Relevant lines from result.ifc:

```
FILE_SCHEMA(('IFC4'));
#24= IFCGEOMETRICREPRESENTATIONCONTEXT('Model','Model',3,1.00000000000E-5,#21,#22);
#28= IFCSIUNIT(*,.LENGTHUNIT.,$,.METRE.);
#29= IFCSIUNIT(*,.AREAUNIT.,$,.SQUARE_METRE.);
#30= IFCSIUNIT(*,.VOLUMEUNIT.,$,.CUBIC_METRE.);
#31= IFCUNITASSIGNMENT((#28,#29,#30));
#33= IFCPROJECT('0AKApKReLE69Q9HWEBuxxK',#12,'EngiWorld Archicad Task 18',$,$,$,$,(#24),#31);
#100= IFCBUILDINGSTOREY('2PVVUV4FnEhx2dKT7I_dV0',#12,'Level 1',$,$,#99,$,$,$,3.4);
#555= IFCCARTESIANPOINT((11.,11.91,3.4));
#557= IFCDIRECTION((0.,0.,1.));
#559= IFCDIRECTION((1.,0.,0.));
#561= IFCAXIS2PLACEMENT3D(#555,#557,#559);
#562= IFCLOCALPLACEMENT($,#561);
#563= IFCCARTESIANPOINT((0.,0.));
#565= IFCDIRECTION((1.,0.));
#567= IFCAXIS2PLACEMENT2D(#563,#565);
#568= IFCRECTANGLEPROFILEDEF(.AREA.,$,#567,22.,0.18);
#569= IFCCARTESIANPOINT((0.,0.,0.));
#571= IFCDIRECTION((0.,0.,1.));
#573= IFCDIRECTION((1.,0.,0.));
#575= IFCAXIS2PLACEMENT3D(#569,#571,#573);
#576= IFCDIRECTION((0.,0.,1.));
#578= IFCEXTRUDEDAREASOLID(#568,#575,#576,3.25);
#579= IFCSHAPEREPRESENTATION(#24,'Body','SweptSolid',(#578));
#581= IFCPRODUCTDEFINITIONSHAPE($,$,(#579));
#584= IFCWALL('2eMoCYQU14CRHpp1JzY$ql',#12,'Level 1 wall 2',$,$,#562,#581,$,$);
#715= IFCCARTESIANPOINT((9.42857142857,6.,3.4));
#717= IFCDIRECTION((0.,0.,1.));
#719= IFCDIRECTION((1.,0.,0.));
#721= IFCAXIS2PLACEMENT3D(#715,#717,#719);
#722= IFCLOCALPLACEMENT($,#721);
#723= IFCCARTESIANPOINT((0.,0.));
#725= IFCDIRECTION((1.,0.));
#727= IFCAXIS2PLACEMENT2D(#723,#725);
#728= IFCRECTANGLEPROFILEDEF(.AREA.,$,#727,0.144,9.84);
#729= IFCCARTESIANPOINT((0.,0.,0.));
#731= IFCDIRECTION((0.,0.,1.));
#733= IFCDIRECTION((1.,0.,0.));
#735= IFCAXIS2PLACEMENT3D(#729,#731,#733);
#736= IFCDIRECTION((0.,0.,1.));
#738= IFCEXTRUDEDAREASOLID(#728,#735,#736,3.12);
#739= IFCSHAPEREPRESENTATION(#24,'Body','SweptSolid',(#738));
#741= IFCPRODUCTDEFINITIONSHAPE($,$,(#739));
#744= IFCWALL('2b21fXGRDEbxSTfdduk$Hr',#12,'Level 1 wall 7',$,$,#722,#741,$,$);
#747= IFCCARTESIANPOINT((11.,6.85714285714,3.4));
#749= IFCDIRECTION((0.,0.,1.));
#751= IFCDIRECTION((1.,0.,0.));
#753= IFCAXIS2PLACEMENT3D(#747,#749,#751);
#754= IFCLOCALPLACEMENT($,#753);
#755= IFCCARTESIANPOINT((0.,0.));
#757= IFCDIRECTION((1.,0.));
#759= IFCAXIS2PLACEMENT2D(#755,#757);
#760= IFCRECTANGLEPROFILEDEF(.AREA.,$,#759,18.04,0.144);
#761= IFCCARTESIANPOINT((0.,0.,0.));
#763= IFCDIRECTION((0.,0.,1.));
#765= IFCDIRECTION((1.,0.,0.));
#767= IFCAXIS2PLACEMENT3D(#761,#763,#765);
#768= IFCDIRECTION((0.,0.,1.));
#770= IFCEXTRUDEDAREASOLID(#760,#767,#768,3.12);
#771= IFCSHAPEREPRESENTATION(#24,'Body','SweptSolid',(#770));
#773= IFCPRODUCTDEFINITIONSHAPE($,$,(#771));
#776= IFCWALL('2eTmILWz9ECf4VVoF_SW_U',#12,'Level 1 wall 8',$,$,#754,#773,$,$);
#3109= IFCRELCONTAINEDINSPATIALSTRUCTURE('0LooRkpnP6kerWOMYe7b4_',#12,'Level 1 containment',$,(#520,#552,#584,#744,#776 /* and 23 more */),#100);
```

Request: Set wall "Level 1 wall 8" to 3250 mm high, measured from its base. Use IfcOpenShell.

```python
import ifcopenshell
import ifcopenshell.geom
import ifcopenshell.util.shape
import ifcopenshell.util.unit

model = ifcopenshell.open("result.ifc")
unit_scale = ifcopenshell.util.unit.calculate_unit_scale(model)
settings = ifcopenshell.geom.settings()


def volume(element):
    """Net volume in cubic metres, openings subtracted."""
    shape = ifcopenshell.geom.create_shape(settings, element)
    return ifcopenshell.util.shape.get_volume(shape.geometry)


wall = model.by_id(776)
before = volume(wall)

body = next(r for r in wall.Representation.Representations if r.RepresentationIdentifier == "Body")
solid = body.Items[0]
old_height = solid.Depth
solid.Depth = 3.25 / unit_scale
after = volume(wall)

print(f"height {old_height:g} -> {solid.Depth:g}, volume {before:.3f} -> {after:.3f} m3")

model.write("result-out.ifc")
```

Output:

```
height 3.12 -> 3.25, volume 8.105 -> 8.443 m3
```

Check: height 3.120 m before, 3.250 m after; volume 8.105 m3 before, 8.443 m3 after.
